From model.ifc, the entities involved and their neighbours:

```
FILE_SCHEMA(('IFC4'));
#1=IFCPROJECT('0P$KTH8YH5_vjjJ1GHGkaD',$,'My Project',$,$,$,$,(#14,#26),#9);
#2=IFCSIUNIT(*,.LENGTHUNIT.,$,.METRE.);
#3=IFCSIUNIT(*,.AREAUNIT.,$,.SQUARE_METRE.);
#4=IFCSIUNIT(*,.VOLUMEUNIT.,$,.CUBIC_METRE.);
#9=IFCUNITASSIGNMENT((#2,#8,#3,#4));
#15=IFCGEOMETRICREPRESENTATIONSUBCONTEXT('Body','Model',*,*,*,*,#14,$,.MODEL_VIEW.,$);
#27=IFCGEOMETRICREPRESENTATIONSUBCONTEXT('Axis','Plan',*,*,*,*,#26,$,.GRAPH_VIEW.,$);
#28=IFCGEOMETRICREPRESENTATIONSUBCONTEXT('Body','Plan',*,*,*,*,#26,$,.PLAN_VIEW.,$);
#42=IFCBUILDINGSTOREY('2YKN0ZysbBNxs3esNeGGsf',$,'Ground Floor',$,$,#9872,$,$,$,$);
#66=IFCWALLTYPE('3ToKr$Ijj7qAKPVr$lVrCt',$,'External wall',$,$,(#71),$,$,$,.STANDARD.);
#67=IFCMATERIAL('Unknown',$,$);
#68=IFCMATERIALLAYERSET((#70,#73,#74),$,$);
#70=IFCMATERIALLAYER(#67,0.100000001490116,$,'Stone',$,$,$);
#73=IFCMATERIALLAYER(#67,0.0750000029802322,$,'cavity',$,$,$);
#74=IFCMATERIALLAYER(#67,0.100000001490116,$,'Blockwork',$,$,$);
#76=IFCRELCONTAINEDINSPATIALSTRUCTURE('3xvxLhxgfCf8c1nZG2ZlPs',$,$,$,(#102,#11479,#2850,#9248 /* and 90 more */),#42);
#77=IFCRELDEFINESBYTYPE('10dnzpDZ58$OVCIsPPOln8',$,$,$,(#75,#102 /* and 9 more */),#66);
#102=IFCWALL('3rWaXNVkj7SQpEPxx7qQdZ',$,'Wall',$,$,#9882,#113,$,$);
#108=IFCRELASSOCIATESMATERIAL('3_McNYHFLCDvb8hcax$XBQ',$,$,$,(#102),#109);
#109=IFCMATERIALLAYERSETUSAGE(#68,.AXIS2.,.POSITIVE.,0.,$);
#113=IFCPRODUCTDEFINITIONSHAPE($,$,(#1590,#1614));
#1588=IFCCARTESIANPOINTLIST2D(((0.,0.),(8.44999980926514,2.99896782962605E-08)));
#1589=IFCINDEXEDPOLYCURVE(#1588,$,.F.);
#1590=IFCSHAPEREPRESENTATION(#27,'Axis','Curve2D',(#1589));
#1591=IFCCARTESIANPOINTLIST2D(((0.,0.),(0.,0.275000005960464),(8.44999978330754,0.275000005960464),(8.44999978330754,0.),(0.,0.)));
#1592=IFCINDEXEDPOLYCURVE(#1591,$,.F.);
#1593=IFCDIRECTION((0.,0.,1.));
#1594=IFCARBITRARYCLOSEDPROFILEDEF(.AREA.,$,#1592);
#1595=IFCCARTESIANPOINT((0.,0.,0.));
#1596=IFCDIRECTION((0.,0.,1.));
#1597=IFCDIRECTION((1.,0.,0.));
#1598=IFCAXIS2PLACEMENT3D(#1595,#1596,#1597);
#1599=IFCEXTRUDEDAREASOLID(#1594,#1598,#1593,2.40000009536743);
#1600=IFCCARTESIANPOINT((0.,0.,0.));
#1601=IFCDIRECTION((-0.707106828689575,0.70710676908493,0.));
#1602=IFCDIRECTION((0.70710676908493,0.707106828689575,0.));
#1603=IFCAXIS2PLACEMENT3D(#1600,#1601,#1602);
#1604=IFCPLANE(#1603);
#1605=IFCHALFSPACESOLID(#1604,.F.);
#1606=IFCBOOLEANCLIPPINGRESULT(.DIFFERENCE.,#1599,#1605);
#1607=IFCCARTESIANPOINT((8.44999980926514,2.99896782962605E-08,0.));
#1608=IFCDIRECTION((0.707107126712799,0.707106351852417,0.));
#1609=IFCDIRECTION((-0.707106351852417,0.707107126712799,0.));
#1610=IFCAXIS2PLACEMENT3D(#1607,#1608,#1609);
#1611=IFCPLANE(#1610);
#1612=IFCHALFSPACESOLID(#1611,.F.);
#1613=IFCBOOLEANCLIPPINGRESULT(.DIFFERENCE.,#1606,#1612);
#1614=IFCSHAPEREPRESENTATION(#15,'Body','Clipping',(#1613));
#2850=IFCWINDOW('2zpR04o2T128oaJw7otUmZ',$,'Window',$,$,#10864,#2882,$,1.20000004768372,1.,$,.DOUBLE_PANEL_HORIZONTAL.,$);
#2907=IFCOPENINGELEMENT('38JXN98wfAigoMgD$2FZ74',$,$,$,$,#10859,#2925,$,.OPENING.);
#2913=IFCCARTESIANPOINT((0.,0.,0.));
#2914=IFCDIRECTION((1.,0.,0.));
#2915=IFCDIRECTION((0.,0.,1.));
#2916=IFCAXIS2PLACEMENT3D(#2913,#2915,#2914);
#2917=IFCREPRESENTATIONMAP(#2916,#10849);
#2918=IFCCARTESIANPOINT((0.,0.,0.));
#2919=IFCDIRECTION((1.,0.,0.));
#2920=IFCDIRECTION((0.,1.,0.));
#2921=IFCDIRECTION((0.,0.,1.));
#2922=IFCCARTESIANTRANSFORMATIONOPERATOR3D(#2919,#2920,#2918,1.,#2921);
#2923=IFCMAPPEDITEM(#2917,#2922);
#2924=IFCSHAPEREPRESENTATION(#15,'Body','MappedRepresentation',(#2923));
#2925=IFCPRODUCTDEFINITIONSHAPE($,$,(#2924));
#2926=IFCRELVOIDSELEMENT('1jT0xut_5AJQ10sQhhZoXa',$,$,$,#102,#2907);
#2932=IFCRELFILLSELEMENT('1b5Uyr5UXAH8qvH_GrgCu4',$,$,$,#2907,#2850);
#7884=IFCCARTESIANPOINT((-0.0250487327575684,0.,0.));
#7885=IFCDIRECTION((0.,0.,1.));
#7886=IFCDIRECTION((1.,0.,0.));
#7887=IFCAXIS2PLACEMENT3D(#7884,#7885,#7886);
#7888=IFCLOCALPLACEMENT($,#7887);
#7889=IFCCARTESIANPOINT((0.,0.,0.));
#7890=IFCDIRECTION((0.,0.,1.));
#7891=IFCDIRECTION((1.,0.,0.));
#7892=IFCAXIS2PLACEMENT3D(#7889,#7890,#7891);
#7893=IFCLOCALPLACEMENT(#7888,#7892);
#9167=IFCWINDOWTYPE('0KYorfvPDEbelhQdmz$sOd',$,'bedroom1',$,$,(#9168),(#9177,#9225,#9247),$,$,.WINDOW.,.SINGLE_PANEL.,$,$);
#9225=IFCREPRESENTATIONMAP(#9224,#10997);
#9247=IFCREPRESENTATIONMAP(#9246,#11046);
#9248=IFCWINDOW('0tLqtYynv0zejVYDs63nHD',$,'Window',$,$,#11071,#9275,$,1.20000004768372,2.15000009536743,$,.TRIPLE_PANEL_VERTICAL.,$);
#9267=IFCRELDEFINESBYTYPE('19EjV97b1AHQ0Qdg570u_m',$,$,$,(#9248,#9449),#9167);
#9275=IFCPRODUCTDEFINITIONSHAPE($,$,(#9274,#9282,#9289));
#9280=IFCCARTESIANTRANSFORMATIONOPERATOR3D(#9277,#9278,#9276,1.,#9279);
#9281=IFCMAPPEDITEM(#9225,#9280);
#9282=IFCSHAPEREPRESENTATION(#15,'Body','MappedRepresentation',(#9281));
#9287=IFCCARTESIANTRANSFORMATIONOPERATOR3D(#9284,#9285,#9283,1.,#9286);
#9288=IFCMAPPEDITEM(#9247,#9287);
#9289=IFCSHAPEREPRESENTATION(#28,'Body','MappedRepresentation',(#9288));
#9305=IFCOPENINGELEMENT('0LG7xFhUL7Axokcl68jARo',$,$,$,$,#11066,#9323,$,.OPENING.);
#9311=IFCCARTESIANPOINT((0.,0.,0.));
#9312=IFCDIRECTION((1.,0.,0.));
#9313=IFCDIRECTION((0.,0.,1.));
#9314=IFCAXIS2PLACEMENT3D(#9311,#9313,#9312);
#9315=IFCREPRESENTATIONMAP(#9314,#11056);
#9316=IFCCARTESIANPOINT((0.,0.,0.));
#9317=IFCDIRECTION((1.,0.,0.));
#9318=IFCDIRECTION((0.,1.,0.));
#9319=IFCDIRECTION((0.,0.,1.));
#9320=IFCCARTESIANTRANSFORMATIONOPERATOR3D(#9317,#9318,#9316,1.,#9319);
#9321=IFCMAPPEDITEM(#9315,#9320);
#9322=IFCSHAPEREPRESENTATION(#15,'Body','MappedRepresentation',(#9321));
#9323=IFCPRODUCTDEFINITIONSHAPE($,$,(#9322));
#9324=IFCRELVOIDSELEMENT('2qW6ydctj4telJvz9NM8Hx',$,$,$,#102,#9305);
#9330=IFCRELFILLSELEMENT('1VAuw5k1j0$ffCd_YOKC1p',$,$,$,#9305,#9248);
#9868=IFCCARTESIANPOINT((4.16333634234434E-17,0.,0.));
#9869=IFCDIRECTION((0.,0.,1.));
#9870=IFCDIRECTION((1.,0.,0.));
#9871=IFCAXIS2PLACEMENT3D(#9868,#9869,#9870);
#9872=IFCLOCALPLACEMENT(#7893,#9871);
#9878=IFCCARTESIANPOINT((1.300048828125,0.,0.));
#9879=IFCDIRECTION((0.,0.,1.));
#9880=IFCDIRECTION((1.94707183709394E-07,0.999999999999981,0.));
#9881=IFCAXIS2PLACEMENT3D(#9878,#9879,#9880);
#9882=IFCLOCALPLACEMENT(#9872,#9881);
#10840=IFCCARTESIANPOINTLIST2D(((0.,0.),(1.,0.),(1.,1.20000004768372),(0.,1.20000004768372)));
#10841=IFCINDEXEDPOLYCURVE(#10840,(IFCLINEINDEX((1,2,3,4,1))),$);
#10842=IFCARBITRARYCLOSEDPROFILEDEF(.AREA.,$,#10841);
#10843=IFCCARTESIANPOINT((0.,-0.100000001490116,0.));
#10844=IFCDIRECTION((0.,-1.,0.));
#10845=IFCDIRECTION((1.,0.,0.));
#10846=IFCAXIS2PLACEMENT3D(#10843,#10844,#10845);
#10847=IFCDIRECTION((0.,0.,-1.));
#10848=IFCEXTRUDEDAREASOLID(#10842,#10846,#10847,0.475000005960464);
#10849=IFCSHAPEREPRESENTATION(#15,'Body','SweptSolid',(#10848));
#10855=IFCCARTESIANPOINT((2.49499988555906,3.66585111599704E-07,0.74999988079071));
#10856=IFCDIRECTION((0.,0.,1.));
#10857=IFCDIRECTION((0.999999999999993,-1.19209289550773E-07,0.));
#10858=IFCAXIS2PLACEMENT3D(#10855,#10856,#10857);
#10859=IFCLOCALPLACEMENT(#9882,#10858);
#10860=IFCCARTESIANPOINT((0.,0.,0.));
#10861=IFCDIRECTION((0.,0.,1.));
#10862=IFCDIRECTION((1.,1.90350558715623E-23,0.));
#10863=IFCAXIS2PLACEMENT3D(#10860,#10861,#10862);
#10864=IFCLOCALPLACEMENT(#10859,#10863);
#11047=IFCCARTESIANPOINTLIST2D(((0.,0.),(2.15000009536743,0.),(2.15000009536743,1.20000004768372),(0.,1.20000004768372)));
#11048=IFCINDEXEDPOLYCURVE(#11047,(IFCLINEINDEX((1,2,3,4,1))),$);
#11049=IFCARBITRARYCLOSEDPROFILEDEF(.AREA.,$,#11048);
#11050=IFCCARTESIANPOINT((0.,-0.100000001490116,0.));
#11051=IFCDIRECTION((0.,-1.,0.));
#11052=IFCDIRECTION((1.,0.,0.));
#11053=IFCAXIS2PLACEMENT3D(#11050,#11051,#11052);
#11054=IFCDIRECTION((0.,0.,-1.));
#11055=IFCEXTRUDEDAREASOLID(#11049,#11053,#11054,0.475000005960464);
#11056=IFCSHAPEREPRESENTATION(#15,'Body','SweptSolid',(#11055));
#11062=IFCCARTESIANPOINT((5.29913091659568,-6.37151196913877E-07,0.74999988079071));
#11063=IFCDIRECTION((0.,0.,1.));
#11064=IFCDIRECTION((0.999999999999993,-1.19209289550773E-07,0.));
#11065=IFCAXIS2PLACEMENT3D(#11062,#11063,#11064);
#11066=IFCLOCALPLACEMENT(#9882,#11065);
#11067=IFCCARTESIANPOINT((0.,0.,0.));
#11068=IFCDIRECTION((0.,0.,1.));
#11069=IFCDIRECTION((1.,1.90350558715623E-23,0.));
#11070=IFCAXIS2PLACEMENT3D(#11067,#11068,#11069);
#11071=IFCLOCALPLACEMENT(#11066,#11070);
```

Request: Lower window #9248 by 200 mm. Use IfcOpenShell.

```python
import numpy as np
import ifcopenshell
import ifcopenshell.api.geometry
import ifcopenshell.util.placement
import ifcopenshell.util.unit

model = ifcopenshell.open("model.ifc")
unit_scale = ifcopenshell.util.unit.calculate_unit_scale(model)

window = model.by_guid("0tLqtYynv0zejVYDs63nHD")
opening = window.FillsVoids[0].RelatingOpeningElement
dz = -0.2

shift = np.array([0.0, 0.0, dz])
# The window is placed relative to its opening, so it follows when the opening moves.
matrix = ifcopenshell.util.placement.get_local_placement(opening.ObjectPlacement)
matrix[:3, 3] += shift
ifcopenshell.api.geometry.edit_object_placement(
    model, product=opening, matrix=matrix, is_si=False, should_transform_children=True
)

print(f"moved by {dz * unit_scale:+.3f} m")

model.write("model_v2.ifc")
```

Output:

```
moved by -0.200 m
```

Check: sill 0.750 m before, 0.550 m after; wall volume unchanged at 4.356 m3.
